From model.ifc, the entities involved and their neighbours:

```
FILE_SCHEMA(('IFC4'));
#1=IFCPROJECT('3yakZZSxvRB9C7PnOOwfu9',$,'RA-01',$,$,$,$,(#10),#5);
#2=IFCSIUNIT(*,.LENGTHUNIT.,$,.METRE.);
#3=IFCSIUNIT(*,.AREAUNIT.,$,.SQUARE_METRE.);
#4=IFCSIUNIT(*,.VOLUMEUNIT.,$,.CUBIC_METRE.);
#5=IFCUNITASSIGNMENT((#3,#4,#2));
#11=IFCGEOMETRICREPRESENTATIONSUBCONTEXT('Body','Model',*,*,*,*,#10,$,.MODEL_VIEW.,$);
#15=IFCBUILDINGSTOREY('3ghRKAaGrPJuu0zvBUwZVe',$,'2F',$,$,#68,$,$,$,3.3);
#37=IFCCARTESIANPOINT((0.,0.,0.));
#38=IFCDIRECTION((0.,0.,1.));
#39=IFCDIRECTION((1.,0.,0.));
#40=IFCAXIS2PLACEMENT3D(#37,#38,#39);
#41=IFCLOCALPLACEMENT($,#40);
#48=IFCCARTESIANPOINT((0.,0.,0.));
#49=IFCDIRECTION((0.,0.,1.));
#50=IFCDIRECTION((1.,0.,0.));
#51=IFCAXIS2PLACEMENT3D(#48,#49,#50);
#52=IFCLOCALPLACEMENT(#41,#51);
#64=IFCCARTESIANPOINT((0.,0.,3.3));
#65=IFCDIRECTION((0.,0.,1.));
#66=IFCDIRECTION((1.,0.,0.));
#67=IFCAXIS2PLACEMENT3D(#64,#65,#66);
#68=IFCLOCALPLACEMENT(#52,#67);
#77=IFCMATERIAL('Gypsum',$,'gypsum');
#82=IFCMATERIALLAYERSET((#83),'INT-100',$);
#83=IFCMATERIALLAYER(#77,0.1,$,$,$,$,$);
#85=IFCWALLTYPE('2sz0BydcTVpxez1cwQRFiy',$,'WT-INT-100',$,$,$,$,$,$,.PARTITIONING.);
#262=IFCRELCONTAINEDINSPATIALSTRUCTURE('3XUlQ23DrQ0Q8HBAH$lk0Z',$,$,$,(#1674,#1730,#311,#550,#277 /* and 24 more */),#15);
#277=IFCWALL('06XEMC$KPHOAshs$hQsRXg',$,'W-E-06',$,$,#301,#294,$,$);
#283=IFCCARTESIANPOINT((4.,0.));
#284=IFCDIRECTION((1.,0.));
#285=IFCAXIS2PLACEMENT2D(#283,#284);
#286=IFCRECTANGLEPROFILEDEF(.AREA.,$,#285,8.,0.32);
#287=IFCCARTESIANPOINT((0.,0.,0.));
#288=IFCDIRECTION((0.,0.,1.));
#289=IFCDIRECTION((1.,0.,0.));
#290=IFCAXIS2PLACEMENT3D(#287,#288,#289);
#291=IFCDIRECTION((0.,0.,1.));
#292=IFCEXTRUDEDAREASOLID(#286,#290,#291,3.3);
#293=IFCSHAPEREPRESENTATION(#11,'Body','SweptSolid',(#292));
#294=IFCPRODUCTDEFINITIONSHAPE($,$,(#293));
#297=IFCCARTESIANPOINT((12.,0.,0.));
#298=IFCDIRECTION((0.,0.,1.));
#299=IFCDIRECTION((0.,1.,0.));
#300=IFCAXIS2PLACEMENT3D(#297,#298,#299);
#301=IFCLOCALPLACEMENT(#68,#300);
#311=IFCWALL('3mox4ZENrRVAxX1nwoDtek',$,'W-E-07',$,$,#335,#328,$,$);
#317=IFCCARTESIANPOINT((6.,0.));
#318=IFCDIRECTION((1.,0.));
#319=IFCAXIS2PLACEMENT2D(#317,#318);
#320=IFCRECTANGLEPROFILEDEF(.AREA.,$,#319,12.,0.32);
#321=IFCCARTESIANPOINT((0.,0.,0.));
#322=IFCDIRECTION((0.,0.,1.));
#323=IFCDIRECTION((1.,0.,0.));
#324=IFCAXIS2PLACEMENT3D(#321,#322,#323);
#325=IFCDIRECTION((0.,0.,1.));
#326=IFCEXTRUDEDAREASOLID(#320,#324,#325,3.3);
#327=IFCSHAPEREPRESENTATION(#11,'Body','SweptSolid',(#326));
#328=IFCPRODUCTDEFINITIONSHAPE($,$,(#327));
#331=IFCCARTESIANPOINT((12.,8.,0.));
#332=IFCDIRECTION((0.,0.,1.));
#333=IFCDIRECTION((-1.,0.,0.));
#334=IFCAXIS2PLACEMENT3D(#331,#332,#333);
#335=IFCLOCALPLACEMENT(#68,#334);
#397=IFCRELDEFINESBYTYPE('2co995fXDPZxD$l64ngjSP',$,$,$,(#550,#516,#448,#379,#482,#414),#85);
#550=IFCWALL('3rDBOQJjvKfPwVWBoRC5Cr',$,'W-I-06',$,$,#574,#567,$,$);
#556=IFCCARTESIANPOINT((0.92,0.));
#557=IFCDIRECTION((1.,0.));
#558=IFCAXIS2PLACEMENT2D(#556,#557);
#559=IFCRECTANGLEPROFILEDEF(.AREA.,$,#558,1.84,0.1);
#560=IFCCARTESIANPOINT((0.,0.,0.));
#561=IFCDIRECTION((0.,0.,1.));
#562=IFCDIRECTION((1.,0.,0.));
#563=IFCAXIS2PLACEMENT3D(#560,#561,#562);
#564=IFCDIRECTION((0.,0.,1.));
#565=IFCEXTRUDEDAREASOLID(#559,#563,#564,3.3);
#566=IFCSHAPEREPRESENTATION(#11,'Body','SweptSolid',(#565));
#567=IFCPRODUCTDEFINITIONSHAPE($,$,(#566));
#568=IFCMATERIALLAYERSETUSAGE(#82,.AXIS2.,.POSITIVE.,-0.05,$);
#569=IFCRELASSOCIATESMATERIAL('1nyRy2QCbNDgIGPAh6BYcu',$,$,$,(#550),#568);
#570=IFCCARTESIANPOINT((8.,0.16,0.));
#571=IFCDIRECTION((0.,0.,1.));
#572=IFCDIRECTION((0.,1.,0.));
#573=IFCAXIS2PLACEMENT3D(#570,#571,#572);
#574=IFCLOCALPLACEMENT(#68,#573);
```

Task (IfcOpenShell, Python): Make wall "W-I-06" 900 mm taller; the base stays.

```python
import ifcopenshell
import ifcopenshell.geom
import ifcopenshell.util.representation
import ifcopenshell.util.shape
import ifcopenshell.util.unit

model = ifcopenshell.open("model.ifc")
unit_scale = ifcopenshell.util.unit.calculate_unit_scale(model)
settings = ifcopenshell.geom.settings()


def volume(element):
    """Net volume in cubic metres, openings subtracted."""
    shape = ifcopenshell.geom.create_shape(settings, element)
    return ifcopenshell.util.shape.get_volume(shape.geometry)


wall = model.by_guid("3rDBOQJjvKfPwVWBoRC5Cr")
before = volume(wall)

body = ifcopenshell.util.representation.get_representation(wall, "Model", "Body")
solid = body.Items[0]
old_height = solid.Depth
solid.Depth += 0.9 / unit_scale
after = volume(wall)

print(f"height {old_height:g} -> {solid.Depth:g}, volume {before:.3f} -> {after:.3f} m3")

model.write("model-out.ifc")
```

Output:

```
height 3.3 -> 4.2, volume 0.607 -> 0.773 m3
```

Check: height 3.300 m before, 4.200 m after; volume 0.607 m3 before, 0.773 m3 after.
